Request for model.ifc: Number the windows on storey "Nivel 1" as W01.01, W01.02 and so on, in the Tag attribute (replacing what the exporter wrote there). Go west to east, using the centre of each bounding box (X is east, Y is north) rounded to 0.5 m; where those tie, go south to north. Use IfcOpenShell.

First a look at what the model holds.

```python
import ifcopenshell
import ifcopenshell.util.element
import ifcopenshell.util.placement

model = ifcopenshell.open("model.ifc")
print(model.schema)
storey = next(s for s in model.by_type("IfcBuildingStorey") if s.Name == "Nivel 1")
windows = [e for e in ifcopenshell.util.element.get_decomposition(storey) if e.is_a("IfcWindow")]
for e in sorted(windows, key=lambda e: e.id()):
    origin = ifcopenshell.util.placement.get_local_placement(e.ObjectPlacement)[:3, 3]
    print(e.id(), e.Tag, e.Name, origin.round(2) + 0.0, sep=" | ")
```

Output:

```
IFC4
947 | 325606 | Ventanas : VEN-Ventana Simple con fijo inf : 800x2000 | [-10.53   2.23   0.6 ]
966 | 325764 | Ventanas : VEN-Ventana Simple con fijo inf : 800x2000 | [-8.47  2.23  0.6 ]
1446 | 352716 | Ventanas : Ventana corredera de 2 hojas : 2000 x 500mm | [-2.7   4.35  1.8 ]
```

```python
import ifcopenshell
import ifcopenshell.geom
import ifcopenshell.util.element
import ifcopenshell.util.shape

model = ifcopenshell.open("model.ifc")
settings = ifcopenshell.geom.settings()
settings.set("use-world-coords", True)


def centre(element):
    shape = ifcopenshell.geom.create_shape(settings, element)
    return ifcopenshell.util.shape.get_bbox_centroid(shape.geometry)


storey = next(s for s in model.by_type("IfcBuildingStorey") if s.Name == "Nivel 1")
windows = [e for e in ifcopenshell.util.element.get_decomposition(storey) if e.is_a("IfcWindow")]

# Insertion points can sit at a corner or the storey origin, so sort by the geometry (in metres).
centres = {e: centre(e) for e in windows}
windows.sort(key=lambda e: (round(centres[e][0] / 0.5), centres[e][1]))

for i, e in enumerate(windows, start=1):
    number = f"W01.{i:02d}"
    e.Tag = number
    print(e.id(), number)

model.write("model-out.ifc")
```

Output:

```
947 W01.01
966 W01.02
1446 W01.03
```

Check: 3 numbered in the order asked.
